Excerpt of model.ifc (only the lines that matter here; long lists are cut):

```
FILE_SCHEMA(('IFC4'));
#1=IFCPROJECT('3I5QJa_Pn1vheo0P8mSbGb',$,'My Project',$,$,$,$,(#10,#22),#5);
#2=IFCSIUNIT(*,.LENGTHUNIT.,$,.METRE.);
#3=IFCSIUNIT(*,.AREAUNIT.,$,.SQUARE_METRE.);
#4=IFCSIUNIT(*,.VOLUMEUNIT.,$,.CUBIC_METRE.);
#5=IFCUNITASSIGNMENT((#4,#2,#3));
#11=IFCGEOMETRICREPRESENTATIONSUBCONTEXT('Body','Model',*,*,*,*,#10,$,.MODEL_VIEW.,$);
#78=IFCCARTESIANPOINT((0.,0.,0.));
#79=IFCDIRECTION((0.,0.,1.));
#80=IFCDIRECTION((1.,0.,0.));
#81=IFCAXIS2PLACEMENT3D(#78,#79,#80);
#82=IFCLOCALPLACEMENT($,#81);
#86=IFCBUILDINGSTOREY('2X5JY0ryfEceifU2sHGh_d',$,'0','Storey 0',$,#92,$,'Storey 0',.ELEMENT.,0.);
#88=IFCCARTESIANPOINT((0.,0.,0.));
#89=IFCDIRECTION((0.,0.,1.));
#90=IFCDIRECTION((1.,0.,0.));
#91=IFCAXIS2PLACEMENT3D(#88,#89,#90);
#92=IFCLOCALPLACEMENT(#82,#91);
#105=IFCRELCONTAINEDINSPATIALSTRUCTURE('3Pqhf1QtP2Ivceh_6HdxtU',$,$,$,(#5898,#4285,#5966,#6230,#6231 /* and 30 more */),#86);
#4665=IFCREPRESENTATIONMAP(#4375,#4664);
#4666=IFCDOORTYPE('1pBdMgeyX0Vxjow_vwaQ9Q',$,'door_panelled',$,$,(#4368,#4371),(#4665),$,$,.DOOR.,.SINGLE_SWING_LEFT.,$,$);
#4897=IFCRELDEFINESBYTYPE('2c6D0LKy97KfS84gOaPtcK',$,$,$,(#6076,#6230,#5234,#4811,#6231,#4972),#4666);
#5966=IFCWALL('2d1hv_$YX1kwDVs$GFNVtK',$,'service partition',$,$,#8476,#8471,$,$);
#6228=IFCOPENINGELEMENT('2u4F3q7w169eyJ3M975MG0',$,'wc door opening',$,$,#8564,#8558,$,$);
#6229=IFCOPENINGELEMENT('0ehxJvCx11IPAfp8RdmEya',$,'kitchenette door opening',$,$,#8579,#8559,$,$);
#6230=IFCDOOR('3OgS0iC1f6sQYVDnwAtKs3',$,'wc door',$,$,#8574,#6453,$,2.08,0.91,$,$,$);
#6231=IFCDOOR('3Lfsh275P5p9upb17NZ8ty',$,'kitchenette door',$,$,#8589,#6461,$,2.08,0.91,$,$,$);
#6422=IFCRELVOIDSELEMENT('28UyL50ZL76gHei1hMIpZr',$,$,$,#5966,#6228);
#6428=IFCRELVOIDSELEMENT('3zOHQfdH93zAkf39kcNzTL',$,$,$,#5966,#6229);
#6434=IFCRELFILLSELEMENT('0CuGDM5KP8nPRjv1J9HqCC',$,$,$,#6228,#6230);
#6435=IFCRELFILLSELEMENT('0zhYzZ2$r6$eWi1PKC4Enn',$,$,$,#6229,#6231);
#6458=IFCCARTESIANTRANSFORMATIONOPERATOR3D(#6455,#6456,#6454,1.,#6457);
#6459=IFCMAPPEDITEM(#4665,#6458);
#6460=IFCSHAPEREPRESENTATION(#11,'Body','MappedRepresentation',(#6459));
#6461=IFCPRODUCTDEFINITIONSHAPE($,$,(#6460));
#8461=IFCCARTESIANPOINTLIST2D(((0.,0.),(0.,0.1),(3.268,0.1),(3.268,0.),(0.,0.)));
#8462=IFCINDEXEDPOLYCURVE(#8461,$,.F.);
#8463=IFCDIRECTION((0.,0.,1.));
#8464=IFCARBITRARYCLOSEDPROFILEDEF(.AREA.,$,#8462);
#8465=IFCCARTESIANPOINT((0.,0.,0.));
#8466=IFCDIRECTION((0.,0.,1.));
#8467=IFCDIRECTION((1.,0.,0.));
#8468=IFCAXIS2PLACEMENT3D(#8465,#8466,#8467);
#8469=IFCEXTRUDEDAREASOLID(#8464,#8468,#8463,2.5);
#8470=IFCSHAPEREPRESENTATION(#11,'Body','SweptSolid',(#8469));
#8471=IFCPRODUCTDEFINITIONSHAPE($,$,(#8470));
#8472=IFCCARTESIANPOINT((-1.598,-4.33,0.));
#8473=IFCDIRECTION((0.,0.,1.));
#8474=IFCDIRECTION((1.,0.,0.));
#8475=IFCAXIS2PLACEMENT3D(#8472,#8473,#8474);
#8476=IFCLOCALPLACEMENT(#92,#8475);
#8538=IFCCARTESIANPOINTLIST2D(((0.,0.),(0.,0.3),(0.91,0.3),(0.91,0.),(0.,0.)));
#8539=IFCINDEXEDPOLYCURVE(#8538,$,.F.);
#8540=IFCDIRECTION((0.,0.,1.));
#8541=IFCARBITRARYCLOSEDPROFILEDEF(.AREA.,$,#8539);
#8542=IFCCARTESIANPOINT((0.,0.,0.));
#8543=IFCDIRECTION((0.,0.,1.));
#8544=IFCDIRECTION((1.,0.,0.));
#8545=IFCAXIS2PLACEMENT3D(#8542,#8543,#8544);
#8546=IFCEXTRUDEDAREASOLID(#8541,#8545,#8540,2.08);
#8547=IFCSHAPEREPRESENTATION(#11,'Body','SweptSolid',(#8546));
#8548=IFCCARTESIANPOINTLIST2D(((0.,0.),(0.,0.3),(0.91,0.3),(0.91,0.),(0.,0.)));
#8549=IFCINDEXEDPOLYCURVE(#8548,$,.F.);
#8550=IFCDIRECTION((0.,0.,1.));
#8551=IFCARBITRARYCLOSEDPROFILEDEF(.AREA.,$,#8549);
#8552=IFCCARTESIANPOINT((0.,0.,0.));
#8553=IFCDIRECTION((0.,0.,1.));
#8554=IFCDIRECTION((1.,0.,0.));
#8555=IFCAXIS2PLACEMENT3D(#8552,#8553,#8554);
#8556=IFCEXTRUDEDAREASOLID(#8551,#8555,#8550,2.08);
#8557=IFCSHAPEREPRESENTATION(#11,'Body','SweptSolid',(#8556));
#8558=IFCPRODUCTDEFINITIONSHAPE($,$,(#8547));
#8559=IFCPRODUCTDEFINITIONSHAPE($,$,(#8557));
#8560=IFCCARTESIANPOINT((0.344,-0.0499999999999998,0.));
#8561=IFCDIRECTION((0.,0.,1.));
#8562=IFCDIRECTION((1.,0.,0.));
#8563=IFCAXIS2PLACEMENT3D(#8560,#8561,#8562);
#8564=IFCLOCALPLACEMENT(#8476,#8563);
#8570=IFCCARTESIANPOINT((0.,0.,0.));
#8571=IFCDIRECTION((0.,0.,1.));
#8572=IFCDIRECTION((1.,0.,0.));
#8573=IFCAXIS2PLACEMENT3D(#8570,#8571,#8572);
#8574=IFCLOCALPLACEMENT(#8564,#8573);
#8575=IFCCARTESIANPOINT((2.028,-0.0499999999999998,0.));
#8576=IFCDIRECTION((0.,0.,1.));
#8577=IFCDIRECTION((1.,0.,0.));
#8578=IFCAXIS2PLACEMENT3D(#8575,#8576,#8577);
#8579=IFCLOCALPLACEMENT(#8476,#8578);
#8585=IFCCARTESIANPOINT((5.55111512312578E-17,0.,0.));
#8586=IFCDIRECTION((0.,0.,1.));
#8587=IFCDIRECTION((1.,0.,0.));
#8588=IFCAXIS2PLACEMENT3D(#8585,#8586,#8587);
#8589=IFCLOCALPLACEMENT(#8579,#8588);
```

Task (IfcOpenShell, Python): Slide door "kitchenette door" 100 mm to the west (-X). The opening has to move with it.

```python
import ifcopenshell
import ifcopenshell.api.geometry
import ifcopenshell.util.placement
import ifcopenshell.util.unit

model = ifcopenshell.open("model.ifc")
unit_scale = ifcopenshell.util.unit.calculate_unit_scale(model)

door = model.by_guid("3Lfsh275P5p9upb17NZ8ty")
opening = door.FillsVoids[0].RelatingOpeningElement
wall = opening.VoidsElements[0].RelatingBuildingElement

wall_matrix = ifcopenshell.util.placement.get_local_placement(wall.ObjectPlacement)
shift = wall_matrix[:3, 0] * -0.1 / unit_scale
before = ifcopenshell.util.placement.get_local_placement(door.ObjectPlacement)[:3, 3].copy()

# The door is placed relative to its opening, so it follows when the opening moves.
matrix = ifcopenshell.util.placement.get_local_placement(opening.ObjectPlacement)
matrix[:3, 3] += shift
ifcopenshell.api.geometry.edit_object_placement(
    model, product=opening, matrix=matrix, is_si=False, should_transform_children=True
)

after = ifcopenshell.util.placement.get_local_placement(door.ObjectPlacement)[:3, 3]
print("door moved by", (after - before).round(3) + 0.0)

model.write("model_edited.ifc")
```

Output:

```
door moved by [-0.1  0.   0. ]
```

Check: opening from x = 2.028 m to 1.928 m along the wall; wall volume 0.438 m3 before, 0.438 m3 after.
